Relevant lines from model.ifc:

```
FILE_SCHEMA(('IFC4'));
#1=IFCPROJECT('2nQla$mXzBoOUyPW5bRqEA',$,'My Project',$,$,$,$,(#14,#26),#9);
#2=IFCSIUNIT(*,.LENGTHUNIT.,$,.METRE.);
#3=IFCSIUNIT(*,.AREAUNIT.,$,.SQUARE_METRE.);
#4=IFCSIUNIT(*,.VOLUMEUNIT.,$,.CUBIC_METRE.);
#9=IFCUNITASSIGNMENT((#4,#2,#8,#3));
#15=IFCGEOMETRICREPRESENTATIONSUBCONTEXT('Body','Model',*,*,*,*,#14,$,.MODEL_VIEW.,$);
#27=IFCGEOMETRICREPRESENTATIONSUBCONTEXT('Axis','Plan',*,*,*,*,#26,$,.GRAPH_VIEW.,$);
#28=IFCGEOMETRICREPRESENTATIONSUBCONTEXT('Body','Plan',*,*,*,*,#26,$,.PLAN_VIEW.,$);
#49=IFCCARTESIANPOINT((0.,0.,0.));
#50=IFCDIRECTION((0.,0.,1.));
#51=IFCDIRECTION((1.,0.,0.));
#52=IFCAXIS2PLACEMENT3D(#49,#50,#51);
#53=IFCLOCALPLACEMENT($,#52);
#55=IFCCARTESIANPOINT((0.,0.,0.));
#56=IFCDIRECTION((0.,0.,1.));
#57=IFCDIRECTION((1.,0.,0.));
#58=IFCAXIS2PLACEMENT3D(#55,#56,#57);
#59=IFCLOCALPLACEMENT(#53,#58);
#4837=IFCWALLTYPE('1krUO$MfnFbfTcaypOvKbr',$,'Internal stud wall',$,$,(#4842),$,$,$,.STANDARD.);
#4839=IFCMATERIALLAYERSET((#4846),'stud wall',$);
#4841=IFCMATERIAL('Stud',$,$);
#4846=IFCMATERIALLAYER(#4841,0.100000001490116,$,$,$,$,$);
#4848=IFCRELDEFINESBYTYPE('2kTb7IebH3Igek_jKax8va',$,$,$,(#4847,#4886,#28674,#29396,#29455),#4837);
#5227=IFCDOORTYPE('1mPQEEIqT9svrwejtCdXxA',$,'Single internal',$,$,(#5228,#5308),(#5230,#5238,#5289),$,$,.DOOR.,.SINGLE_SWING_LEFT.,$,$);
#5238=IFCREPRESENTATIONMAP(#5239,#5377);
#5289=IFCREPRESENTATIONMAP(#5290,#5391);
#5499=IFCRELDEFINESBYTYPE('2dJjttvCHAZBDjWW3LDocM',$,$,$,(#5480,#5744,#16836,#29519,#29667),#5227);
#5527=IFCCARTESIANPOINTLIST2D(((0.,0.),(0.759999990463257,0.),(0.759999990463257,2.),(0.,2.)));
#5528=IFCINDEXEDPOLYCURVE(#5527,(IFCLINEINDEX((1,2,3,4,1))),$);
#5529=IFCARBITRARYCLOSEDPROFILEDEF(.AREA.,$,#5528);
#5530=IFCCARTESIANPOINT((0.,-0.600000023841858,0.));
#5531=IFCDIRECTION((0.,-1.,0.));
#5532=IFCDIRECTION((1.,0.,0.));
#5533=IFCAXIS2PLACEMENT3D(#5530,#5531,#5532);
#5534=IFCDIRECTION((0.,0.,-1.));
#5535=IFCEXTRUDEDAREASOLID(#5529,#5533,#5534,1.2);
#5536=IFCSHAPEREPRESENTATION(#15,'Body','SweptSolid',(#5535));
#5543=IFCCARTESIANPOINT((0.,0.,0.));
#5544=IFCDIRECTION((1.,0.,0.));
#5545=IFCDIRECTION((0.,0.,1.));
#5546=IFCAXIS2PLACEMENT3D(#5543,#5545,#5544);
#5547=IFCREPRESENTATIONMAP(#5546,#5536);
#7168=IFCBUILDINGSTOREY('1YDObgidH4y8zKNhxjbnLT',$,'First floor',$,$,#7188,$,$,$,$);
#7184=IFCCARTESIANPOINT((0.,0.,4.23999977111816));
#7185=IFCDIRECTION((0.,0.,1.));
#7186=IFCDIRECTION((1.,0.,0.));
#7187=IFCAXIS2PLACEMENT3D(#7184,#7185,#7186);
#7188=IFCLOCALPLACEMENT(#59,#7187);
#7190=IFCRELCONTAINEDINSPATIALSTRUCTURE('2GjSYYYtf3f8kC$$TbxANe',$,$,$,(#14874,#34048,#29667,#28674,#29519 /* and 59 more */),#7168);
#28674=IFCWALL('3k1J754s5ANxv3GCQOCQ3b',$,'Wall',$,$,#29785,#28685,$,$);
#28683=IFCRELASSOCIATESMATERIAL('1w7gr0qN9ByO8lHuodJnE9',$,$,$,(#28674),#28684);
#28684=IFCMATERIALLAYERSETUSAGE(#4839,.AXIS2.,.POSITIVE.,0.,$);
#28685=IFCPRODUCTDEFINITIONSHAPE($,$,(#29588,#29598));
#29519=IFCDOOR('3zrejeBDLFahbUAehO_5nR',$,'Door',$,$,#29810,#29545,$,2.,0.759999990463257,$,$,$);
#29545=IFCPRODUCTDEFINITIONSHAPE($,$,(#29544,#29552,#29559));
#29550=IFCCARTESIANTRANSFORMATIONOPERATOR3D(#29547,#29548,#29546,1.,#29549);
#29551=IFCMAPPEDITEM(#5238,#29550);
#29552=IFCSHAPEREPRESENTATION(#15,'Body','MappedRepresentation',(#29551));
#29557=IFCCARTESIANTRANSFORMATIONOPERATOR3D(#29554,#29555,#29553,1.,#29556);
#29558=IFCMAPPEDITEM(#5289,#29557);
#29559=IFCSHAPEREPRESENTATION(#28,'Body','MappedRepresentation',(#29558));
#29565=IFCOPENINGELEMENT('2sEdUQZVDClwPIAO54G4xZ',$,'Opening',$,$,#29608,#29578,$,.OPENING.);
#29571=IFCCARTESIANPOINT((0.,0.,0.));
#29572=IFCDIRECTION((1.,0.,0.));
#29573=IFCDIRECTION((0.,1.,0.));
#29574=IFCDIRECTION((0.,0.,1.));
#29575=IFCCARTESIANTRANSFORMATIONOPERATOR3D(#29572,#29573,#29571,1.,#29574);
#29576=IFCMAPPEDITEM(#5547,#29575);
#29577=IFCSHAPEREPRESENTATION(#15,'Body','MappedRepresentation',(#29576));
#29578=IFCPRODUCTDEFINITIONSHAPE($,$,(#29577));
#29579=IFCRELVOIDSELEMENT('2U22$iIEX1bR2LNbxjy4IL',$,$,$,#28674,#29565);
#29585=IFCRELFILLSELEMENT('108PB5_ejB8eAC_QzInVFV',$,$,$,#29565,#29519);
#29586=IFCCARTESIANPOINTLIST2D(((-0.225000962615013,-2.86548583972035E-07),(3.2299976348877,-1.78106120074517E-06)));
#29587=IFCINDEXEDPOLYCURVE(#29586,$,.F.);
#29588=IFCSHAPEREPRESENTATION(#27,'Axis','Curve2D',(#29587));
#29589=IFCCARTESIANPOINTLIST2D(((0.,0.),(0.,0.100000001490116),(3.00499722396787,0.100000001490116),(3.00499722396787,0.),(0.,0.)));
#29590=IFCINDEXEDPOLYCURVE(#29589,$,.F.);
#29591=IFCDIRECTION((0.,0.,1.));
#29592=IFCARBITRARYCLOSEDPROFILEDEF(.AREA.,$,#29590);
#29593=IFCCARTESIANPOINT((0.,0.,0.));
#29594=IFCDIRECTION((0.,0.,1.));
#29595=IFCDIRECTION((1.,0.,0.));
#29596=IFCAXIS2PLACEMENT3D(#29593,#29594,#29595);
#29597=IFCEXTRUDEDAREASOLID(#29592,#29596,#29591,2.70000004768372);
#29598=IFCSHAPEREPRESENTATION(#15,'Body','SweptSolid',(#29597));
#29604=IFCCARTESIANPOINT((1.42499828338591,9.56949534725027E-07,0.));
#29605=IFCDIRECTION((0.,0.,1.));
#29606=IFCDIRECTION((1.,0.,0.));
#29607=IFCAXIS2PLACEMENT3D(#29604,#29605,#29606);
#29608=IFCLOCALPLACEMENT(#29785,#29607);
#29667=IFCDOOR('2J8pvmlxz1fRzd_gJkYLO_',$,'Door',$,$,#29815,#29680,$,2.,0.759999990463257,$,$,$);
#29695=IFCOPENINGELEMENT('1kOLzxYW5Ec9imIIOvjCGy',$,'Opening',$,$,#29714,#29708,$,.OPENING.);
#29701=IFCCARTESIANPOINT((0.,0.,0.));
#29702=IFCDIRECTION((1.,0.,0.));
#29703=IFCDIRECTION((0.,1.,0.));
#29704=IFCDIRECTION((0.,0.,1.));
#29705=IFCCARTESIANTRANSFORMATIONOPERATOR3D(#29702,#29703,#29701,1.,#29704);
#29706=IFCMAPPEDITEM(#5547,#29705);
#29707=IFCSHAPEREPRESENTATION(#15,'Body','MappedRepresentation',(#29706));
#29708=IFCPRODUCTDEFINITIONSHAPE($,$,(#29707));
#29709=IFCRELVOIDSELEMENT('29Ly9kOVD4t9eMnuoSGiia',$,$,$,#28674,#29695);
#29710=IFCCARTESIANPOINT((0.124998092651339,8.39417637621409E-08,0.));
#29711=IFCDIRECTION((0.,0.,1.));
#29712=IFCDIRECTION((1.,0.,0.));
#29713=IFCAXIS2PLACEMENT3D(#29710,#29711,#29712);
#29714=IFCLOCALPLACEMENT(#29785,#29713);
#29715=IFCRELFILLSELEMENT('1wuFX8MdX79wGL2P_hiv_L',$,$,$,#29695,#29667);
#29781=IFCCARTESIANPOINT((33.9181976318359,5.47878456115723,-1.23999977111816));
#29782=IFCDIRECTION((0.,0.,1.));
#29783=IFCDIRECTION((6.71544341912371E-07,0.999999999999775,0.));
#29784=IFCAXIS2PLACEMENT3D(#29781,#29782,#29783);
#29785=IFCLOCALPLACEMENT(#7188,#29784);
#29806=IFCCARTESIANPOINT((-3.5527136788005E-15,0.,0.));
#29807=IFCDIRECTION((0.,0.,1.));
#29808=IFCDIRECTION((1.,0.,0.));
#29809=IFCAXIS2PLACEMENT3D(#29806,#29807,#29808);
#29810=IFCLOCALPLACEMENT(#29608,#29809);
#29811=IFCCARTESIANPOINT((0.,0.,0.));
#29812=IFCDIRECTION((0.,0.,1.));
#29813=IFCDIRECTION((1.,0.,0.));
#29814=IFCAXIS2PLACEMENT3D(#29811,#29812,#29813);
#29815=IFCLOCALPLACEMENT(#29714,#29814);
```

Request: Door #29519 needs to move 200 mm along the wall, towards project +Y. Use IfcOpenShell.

```python
import ifcopenshell
import ifcopenshell.api.geometry
import ifcopenshell.util.placement
import ifcopenshell.util.unit

model = ifcopenshell.open("model.ifc")
unit_scale = ifcopenshell.util.unit.calculate_unit_scale(model)

door = model.by_id(29519)
opening = door.FillsVoids[0].RelatingOpeningElement
wall = opening.VoidsElements[0].RelatingBuildingElement

wall_matrix = ifcopenshell.util.placement.get_local_placement(wall.ObjectPlacement)
shift = wall_matrix[:3, 0] * 0.2 / unit_scale
before = ifcopenshell.util.placement.get_local_placement(door.ObjectPlacement)[:3, 3].copy()

# The door is placed relative to its opening, so it follows when the opening moves.
matrix = ifcopenshell.util.placement.get_local_placement(opening.ObjectPlacement)
matrix[:3, 3] += shift
ifcopenshell.api.geometry.edit_object_placement(
    model, product=opening, matrix=matrix, is_si=False, should_transform_children=True
)

after = ifcopenshell.util.placement.get_local_placement(door.ObjectPlacement)[:3, 3]
print("door moved by", (after - before).round(3) + 0.0)

model.write("model_updated.ifc")
```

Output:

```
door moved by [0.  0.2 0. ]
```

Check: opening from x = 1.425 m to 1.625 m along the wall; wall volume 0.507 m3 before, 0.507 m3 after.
